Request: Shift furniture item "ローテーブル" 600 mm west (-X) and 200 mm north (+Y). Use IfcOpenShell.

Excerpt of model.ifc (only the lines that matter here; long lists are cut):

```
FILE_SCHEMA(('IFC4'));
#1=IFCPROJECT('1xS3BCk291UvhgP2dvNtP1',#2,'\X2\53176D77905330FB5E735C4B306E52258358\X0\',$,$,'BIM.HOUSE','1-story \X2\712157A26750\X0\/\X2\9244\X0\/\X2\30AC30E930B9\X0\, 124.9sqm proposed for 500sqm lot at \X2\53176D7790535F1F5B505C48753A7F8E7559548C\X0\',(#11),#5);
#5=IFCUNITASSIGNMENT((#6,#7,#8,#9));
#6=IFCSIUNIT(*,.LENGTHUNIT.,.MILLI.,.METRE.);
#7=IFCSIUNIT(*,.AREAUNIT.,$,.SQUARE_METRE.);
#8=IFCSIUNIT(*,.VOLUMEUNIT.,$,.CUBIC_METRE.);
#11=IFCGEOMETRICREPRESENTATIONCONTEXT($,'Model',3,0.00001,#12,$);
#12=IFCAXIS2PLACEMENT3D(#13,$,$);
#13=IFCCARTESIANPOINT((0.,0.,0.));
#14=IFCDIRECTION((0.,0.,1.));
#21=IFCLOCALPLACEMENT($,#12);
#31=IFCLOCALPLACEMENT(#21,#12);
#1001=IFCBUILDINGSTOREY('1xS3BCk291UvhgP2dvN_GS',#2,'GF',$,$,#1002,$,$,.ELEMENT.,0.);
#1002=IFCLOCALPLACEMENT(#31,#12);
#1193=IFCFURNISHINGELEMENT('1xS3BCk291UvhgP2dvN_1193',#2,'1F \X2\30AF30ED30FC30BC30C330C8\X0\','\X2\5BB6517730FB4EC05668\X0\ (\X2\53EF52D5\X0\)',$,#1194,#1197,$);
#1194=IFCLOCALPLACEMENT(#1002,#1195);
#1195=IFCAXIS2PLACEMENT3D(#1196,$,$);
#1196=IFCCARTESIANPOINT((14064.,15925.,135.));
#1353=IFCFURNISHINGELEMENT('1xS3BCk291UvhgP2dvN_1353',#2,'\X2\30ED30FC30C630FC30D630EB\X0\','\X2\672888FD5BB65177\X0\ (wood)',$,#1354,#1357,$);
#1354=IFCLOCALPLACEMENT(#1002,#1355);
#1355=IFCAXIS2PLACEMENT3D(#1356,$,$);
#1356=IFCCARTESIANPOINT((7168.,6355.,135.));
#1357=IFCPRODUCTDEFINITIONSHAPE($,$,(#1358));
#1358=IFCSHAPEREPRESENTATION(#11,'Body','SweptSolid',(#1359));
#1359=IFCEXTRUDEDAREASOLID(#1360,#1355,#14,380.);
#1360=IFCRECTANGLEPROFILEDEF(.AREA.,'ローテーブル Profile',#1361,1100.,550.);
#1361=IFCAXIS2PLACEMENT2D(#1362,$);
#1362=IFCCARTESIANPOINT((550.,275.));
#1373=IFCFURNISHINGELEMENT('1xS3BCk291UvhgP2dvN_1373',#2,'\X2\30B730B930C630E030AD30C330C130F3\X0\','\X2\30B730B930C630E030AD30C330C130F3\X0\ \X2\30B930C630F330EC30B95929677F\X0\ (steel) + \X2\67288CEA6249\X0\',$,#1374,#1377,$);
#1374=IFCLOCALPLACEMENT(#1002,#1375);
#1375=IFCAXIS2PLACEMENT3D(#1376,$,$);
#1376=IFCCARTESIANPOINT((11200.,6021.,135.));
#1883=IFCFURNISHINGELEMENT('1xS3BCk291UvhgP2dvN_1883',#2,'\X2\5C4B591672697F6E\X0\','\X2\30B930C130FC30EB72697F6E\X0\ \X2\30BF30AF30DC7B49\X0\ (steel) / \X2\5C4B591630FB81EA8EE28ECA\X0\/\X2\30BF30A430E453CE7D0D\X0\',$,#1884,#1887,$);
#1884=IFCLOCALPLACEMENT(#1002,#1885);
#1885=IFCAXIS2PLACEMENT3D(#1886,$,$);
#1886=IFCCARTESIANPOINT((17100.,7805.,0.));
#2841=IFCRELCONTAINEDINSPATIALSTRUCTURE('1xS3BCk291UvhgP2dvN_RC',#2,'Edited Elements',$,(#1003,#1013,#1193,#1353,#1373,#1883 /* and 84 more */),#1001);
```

```python
import ifcopenshell
import ifcopenshell.api.geometry
import ifcopenshell.util.placement

model = ifcopenshell.open("model.ifc")

item = model.by_id(1353)
matrix = ifcopenshell.util.placement.get_local_placement(item.ObjectPlacement)
matrix[0, 3] -= 600.0
matrix[1, 3] += 200.0
ifcopenshell.api.geometry.edit_object_placement(model, product=item, matrix=matrix, is_si=False)

print(ifcopenshell.util.placement.get_local_placement(item.ObjectPlacement).round(3) + 0.0)

model.write("model_v2.ifc")
```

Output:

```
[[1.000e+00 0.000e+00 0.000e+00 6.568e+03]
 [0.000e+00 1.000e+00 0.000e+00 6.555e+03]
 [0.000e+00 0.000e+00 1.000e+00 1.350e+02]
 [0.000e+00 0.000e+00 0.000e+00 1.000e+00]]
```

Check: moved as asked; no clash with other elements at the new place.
